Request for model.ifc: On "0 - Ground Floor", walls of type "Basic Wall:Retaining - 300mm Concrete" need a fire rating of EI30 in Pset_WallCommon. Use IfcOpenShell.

First a look at what the model holds.

```python
import ifcopenshell
import ifcopenshell.util.element

model = ifcopenshell.open("model.ifc")
print(model.schema)
storey = next(s for s in model.by_type("IfcBuildingStorey") if s.Name == "0 - Ground Floor")
walls = [e for e in ifcopenshell.util.element.get_decomposition(storey) if e.is_a("IfcWall")]
seen = {}
for e in walls:
    element_type = ifcopenshell.util.element.get_type(e)
    key = (element_type.Name if element_type != e and element_type else None, ifcopenshell.util.element.get_pset(e, "Pset_WallCommon", "FireRating"))
    seen[key] = seen.get(key, 0) + 1
for (name, value), count in sorted(seen.items(), key=str):
    print(count, "x", name, "|", value)
```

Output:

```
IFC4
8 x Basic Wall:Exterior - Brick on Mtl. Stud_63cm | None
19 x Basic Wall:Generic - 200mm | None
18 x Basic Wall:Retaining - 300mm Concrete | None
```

```python
import ifcopenshell
import ifcopenshell.api.pset
import ifcopenshell.util.element

model = ifcopenshell.open("model.ifc")

storey = next(s for s in model.by_type("IfcBuildingStorey") if s.Name == "0 - Ground Floor")
walls = [e for e in ifcopenshell.util.element.get_decomposition(storey) if e.is_a("IfcWall")]

count = 0
for e in walls:
    element_type = ifcopenshell.util.element.get_type(e)
    if element_type in (None, e) or element_type.Name != "Basic Wall:Retaining - 300mm Concrete":
        continue
    # add_pset returns the element's existing set when there is one.
    pset = ifcopenshell.api.pset.add_pset(model, product=e, name="Pset_WallCommon")
    ifcopenshell.api.pset.edit_pset(model, pset=pset, properties={"FireRating": "EI30"})
    count += 1

print(count, "walls updated")

model.write("model_edited.ifc")
```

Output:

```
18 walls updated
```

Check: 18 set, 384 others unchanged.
